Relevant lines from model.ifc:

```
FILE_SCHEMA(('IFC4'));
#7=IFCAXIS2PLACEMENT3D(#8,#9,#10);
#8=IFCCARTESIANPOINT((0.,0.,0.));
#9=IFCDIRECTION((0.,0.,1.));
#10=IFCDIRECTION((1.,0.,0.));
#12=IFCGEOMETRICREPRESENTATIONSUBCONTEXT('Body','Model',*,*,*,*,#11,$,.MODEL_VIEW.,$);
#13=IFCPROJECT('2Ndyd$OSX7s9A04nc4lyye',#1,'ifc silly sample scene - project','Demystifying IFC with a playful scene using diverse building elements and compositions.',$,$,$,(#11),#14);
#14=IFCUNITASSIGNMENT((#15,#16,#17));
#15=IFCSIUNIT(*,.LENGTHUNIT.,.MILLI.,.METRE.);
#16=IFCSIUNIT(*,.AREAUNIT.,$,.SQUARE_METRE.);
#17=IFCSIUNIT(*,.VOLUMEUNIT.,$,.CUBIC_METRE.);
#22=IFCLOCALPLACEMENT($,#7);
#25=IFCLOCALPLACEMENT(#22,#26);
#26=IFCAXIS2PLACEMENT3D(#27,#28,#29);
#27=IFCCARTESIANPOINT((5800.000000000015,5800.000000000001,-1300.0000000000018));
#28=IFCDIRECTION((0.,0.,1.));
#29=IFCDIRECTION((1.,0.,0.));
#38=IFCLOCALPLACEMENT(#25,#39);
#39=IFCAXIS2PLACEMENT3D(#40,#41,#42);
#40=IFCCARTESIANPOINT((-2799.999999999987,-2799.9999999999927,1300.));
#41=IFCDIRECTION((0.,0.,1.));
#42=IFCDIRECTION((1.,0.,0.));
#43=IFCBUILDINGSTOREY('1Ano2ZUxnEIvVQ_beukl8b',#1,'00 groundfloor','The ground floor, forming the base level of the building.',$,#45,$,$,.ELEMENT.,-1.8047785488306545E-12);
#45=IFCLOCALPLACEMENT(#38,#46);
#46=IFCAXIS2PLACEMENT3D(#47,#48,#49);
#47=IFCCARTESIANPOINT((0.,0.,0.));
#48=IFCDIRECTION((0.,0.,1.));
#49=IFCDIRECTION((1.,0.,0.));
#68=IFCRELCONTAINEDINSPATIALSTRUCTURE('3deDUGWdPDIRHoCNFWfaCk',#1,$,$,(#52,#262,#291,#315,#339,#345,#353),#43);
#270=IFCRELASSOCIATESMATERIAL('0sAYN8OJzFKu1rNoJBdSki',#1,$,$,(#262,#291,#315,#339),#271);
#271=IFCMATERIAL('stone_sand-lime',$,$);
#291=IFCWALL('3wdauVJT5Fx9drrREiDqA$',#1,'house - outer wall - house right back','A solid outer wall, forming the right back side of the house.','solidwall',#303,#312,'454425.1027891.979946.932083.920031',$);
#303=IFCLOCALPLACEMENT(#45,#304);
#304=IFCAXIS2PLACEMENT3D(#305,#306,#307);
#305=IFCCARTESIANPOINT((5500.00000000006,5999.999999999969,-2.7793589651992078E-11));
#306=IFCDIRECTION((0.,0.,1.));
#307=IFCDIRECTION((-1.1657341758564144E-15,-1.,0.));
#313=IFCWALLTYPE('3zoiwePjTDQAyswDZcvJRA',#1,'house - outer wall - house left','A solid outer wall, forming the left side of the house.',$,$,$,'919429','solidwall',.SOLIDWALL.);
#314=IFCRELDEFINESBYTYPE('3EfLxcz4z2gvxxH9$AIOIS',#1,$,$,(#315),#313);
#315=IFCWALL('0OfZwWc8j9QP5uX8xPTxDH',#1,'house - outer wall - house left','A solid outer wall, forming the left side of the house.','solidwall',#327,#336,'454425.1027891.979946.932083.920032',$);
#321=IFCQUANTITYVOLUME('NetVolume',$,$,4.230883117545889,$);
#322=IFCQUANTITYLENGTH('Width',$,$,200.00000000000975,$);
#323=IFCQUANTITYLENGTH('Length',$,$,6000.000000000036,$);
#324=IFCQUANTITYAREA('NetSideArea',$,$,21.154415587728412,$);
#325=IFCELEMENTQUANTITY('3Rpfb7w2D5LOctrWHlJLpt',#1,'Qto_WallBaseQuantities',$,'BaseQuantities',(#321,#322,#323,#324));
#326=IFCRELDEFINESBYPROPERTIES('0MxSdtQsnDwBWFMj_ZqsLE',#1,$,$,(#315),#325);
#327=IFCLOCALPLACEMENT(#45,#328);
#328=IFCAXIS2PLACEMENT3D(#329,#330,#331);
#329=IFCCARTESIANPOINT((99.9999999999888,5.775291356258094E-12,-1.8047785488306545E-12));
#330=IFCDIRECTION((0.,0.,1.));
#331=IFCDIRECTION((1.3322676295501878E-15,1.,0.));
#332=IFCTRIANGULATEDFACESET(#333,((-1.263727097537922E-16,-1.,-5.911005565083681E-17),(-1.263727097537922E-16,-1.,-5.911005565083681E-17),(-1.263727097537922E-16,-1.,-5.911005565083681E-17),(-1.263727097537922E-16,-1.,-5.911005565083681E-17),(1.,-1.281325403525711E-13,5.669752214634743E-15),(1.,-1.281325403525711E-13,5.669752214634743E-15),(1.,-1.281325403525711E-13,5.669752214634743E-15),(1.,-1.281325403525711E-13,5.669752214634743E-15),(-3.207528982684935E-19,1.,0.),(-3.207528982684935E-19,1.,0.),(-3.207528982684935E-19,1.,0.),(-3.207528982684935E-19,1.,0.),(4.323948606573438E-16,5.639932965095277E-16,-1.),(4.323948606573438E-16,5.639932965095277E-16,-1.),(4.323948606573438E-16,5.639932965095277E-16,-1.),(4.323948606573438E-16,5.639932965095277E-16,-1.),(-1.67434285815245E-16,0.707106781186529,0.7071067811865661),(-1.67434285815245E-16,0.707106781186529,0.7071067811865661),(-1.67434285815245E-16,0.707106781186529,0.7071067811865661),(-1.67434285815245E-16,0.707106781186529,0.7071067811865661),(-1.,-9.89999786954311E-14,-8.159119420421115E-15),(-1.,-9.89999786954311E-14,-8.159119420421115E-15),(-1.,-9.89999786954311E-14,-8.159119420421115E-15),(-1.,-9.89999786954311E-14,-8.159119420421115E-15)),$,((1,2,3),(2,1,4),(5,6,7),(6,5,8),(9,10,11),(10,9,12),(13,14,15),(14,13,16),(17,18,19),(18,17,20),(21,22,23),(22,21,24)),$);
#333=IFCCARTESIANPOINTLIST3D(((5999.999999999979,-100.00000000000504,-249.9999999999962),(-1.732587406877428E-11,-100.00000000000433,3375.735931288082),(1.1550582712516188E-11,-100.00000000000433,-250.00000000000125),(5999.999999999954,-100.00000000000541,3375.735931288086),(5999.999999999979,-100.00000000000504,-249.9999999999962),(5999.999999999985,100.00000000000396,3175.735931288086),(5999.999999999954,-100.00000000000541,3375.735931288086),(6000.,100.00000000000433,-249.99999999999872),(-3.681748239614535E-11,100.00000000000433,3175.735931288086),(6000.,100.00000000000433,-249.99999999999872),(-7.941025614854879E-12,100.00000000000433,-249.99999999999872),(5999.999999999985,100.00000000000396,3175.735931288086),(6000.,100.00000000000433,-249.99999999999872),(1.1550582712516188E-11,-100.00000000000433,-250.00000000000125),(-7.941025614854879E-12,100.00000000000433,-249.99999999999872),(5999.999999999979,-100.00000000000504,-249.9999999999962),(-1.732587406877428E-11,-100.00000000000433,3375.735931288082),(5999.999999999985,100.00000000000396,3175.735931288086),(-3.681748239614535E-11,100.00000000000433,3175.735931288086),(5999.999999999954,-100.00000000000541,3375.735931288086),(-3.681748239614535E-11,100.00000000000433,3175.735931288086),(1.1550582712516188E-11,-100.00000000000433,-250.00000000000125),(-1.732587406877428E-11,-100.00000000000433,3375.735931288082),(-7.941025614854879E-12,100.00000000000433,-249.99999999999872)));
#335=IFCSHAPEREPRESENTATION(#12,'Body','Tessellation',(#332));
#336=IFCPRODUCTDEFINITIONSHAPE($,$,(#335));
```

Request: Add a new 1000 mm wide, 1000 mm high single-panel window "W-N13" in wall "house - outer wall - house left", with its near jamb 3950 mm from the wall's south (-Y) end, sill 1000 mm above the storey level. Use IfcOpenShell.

```python
import numpy as np
import ifcopenshell
import ifcopenshell.api.feature
import ifcopenshell.api.geometry
import ifcopenshell.api.pset
import ifcopenshell.api.root
import ifcopenshell.api.spatial
import ifcopenshell.geom
import ifcopenshell.util.element
import ifcopenshell.util.placement
import ifcopenshell.util.representation
import ifcopenshell.util.shape
import ifcopenshell.util.unit

model = ifcopenshell.open("model.ifc")
unit_scale = ifcopenshell.util.unit.calculate_unit_scale(model)
area_scale = ifcopenshell.util.unit.calculate_unit_scale(model, "AREAUNIT")
volume_scale = ifcopenshell.util.unit.calculate_unit_scale(model, "VOLUMEUNIT")
settings = ifcopenshell.geom.settings()


def volume(element):
    """Net volume in cubic metres, openings subtracted."""
    shape = ifcopenshell.geom.create_shape(settings, element)
    return ifcopenshell.util.shape.get_volume(shape.geometry)


wall = model.by_guid("0OfZwWc8j9QP5uX8xPTxDH")
storey = ifcopenshell.util.element.get_container(wall, ifc_class="IfcBuildingStorey")
context = ifcopenshell.util.representation.get_context(model, "Model", "Body", "MODEL_VIEW")
before = volume(wall)

width, height, from_end, sill = 1, 1, 3.95, 1  # metres

# The wall runs along its own X axis, and the end named is its -X end.
wall_shape = ifcopenshell.geom.create_shape(settings, wall)
x, y, z = ifcopenshell.util.shape.get_vertices(wall_shape.geometry).T
start = x.min() + from_end
face, thickness = float(y.min()), float(y.max() - y.min())
wall_matrix = ifcopenshell.util.placement.get_local_placement(wall.ObjectPlacement)
level = ifcopenshell.util.placement.get_local_placement(storey.ObjectPlacement)[2, 3]


def in_wall(x, y):
    """Placement at x, y metres in the wall's axes, at sill height."""
    matrix = wall_matrix.copy()
    matrix[:, 3] = wall_matrix @ np.array([x / unit_scale, y / unit_scale, 0.0, 1.0])
    matrix[2, 3] = level + sill / unit_scale
    return matrix


# Opening: a box that overshoots both wall faces by 50 mm.
opening = ifcopenshell.api.root.create_entity(model, ifc_class="IfcOpeningElement", predefined_type="OPENING")
box = ifcopenshell.api.geometry.add_wall_representation(
    model, context=context, length=width, height=height, thickness=thickness + 0.1
)
ifcopenshell.api.geometry.assign_representation(model, product=opening, representation=box)
ifcopenshell.api.geometry.edit_object_placement(model, product=opening, matrix=in_wall(start, face - 0.05), is_si=False)
ifcopenshell.api.feature.add_feature(model, feature=opening, element=wall)

window = ifcopenshell.api.root.create_entity(model, ifc_class="IfcWindow", name="W-N13", predefined_type="WINDOW")
window.OverallWidth, window.OverallHeight = width / unit_scale, height / unit_scale
window.PartitioningType = "SINGLE_PANEL"
body = ifcopenshell.api.geometry.add_window_representation(
    model,
    context=context,
    overall_width=window.OverallWidth,
    overall_height=window.OverallHeight,
    partition_type="SINGLE_PANEL",
)
ifcopenshell.api.geometry.assign_representation(model, product=window, representation=body)
ifcopenshell.api.spatial.assign_container(model, products=[window], relating_structure=storey)
ifcopenshell.api.feature.add_filling(model, opening=opening, element=window)

# Centre the window in the wall's thickness.
ifcopenshell.api.geometry.edit_object_placement(model, product=window, matrix=in_wall(start, face), is_si=False)
window_shape = ifcopenshell.geom.create_shape(settings, window)
depth = ifcopenshell.util.shape.get_vertices(window_shape.geometry)[:, 1]
offset = face + thickness / 2 - (depth.min() + depth.max()) / 2
ifcopenshell.api.geometry.edit_object_placement(model, product=window, matrix=in_wall(start, offset), is_si=False)

after = volume(wall)

# Update the wall's stored quantities.
qto = model.by_id(ifcopenshell.util.element.get_pset(wall, "Qto_WallBaseQuantities", should_inherit=False)["id"])
ifcopenshell.api.pset.edit_qto(model, qto=qto, properties={
    "NetVolume": after / volume_scale,
    "NetSideArea": after / thickness / area_scale,
})

print(f"wall volume {before:.3f} -> {after:.3f} m3")

model.write("model_edited.ifc")
```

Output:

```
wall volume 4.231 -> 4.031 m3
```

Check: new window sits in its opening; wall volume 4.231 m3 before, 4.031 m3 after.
